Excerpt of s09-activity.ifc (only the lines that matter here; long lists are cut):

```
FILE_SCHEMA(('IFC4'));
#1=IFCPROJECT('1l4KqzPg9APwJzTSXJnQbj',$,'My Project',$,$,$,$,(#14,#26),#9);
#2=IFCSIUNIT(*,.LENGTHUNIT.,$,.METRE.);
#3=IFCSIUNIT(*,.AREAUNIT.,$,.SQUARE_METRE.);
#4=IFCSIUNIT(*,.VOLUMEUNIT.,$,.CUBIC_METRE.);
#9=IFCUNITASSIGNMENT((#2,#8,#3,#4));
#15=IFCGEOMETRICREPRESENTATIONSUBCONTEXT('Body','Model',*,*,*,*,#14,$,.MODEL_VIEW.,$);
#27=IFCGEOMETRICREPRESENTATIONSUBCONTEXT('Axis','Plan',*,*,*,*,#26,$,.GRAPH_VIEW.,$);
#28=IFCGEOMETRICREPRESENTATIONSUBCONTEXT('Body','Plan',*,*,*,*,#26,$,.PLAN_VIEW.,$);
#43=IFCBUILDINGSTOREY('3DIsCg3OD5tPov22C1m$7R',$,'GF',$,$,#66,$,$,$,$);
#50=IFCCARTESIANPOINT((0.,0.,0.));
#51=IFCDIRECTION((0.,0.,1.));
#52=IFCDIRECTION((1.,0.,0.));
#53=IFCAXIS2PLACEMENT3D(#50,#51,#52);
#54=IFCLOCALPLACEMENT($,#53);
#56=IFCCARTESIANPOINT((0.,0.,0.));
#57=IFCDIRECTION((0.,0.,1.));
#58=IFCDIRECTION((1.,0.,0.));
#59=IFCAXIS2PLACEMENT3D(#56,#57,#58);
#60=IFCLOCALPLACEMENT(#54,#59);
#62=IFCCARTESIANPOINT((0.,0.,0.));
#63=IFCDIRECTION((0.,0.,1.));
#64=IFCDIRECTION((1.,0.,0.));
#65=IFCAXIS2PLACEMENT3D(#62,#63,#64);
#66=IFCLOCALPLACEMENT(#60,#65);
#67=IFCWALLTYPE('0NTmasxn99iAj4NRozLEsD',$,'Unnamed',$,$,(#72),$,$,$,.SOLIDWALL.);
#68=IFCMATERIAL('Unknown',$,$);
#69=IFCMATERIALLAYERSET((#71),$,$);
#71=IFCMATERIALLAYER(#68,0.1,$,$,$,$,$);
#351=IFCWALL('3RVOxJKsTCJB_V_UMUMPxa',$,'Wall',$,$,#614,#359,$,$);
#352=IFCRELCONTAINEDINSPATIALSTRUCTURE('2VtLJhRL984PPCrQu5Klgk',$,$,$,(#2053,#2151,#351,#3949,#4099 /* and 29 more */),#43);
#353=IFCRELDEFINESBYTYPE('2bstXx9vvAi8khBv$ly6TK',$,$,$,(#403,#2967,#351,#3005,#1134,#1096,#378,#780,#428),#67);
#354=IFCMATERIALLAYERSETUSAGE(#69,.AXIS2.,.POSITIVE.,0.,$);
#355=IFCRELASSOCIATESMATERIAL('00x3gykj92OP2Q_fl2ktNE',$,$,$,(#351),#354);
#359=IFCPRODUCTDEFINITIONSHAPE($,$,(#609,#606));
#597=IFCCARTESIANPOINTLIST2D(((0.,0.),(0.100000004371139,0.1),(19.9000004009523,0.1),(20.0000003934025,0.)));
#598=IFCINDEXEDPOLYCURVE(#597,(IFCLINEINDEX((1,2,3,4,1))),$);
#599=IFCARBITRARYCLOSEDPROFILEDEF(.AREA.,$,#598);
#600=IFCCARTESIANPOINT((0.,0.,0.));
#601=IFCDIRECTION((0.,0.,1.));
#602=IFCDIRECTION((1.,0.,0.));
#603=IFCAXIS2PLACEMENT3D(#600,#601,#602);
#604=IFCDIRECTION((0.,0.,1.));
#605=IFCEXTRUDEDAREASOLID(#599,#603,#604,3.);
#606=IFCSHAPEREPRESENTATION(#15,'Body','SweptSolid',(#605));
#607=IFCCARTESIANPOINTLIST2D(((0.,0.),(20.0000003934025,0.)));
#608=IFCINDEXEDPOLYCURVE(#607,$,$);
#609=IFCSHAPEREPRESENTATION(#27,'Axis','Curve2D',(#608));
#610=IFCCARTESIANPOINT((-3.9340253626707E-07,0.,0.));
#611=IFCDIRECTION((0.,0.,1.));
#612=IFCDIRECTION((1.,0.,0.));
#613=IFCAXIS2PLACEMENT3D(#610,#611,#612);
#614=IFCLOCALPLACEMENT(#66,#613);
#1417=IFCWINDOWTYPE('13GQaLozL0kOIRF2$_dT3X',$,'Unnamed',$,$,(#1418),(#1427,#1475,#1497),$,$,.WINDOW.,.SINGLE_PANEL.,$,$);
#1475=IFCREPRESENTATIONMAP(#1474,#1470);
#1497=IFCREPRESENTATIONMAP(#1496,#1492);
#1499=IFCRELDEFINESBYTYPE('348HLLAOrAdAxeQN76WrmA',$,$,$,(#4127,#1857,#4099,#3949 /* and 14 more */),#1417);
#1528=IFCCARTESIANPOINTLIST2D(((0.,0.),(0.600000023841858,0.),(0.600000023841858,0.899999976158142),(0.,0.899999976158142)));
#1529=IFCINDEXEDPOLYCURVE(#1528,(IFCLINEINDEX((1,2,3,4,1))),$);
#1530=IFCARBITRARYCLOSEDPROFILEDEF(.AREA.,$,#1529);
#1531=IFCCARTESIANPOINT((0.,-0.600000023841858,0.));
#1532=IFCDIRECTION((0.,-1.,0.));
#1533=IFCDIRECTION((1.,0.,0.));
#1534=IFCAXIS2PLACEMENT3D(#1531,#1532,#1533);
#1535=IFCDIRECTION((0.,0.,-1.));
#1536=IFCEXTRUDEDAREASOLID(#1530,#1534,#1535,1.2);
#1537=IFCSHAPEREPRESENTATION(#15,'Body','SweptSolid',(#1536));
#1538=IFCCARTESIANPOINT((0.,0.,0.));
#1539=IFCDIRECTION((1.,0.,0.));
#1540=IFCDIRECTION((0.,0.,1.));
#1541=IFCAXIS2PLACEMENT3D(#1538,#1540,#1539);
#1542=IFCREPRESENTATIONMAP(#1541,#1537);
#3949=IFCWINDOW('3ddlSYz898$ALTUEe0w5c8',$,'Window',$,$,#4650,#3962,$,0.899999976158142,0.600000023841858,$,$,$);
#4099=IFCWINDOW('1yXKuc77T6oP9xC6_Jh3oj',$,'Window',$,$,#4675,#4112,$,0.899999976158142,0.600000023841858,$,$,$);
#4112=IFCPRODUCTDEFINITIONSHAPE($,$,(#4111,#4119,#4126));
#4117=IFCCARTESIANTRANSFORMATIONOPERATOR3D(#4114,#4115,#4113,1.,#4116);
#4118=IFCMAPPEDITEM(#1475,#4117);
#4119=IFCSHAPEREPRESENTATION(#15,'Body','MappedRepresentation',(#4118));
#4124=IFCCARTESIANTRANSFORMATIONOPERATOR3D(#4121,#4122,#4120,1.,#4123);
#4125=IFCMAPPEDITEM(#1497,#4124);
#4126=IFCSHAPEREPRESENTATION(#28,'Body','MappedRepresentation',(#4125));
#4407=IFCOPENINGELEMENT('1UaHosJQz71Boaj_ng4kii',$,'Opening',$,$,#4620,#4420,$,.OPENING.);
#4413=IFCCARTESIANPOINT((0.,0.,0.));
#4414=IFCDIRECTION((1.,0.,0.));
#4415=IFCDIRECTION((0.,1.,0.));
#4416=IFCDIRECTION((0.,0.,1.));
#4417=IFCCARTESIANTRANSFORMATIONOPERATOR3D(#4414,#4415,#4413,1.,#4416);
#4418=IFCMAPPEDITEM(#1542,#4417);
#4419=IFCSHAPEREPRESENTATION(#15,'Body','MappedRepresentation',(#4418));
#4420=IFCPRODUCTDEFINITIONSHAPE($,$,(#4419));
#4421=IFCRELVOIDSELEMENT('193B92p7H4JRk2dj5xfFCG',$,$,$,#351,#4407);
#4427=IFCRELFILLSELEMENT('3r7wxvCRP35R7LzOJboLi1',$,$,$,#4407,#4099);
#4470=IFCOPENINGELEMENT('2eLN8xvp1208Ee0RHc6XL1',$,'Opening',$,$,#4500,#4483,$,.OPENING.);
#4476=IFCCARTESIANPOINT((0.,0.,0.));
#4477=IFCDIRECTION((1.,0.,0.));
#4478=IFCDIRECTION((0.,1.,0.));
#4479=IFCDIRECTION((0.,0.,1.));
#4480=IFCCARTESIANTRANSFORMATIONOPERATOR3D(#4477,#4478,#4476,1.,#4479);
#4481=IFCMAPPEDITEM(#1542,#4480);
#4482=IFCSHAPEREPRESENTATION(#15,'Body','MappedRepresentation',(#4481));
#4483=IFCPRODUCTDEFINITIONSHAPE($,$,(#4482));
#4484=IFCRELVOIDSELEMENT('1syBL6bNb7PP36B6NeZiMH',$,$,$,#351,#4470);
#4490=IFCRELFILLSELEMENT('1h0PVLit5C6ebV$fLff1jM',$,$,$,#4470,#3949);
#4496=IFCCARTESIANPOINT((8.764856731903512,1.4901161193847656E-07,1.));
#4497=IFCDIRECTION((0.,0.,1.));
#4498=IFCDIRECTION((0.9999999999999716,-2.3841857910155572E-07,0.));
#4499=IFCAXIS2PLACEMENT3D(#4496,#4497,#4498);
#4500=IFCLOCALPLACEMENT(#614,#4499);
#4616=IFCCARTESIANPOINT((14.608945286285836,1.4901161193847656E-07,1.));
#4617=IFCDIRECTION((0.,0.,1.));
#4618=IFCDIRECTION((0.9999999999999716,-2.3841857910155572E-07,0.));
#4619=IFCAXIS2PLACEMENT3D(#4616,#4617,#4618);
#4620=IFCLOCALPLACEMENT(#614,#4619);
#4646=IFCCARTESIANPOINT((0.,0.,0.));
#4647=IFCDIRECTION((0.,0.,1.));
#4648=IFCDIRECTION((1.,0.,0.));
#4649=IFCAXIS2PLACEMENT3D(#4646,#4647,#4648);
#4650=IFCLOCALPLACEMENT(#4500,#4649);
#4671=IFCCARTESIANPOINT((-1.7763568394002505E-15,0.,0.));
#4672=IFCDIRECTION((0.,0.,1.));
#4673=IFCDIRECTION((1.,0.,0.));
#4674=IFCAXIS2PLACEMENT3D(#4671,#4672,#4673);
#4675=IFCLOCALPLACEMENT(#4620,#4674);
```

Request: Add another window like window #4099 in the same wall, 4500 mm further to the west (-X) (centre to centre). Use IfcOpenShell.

```python
import ifcopenshell
import ifcopenshell.api.feature
import ifcopenshell.api.geometry
import ifcopenshell.api.root
import ifcopenshell.geom
import ifcopenshell.util.element
import ifcopenshell.util.placement
import ifcopenshell.util.shape
import ifcopenshell.util.unit

model = ifcopenshell.open("s09-activity.ifc")
unit_scale = ifcopenshell.util.unit.calculate_unit_scale(model)
settings = ifcopenshell.geom.settings()


def volume(element):
    """Net volume in cubic metres, openings subtracted."""
    shape = ifcopenshell.geom.create_shape(settings, element)
    return ifcopenshell.util.shape.get_volume(shape.geometry)


window = model.by_guid("1yXKuc77T6oP9xC6_Jh3oj")
opening = window.FillsVoids[0].RelatingOpeningElement
wall = opening.VoidsElements[0].RelatingBuildingElement
before = volume(wall)
shift = ifcopenshell.util.placement.get_local_placement(wall.ObjectPlacement)[:3, 0] * -4.5 / unit_scale

# copy_class copies the void relationship, type, container and properties, but no geometry.
new_opening = ifcopenshell.api.root.copy_class(model, product=opening)
new_opening.Representation = ifcopenshell.util.element.copy_deep(
    model, opening.Representation, exclude=["IfcGeometricRepresentationContext", "IfcRepresentationMap"]
)
new_window = ifcopenshell.api.root.copy_class(model, product=window)
new_window.Representation = ifcopenshell.util.element.copy_deep(
    model, window.Representation, exclude=["IfcGeometricRepresentationContext", "IfcRepresentationMap"]
)
ifcopenshell.api.feature.add_filling(model, opening=new_opening, element=new_window)

for old, new in ((opening, new_opening), (window, new_window)):
    matrix = ifcopenshell.util.placement.get_local_placement(old.ObjectPlacement)
    matrix[:3, 3] += shift
    ifcopenshell.api.geometry.edit_object_placement(model, product=new, matrix=matrix, is_si=False)

after = volume(wall)

print(f"wall volume {before:.3f} -> {after:.3f} m3")

model.write("s09-activity_rev.ifc")
```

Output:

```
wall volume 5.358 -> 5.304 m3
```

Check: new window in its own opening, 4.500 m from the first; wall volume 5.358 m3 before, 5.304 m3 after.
